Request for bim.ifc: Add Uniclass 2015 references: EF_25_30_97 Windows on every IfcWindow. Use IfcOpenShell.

First a look at what the model holds.

```python
import ifcopenshell

model = ifcopenshell.open("bim.ifc")
print(model.schema)
print("classifications:", [c.Name for c in model.by_type("IfcClassification")])
for ifc_class in ("IfcDoor", "IfcRoof", "IfcStair", "IfcWall", "IfcWindow"):
    print(ifc_class, len(model.by_type(ifc_class)))
```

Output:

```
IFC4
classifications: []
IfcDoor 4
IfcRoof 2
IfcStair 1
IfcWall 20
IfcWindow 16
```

```python
import ifcopenshell
import ifcopenshell.api.classification

model = ifcopenshell.open("bim.ifc")

system = ifcopenshell.api.classification.add_classification(model, classification="Uniclass 2015")

codes = {
    "IfcWindow": ("EF_25_30_97", "Windows"),
}
for ifc_class, (code, name) in codes.items():
    products = model.by_type(ifc_class)
    ifcopenshell.api.classification.add_reference(
        model, products=products, classification=system, identification=code, name=name
    )
    print(code, len(products))

model.write("bim_rev.ifc")
```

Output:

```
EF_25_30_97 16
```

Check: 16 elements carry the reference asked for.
